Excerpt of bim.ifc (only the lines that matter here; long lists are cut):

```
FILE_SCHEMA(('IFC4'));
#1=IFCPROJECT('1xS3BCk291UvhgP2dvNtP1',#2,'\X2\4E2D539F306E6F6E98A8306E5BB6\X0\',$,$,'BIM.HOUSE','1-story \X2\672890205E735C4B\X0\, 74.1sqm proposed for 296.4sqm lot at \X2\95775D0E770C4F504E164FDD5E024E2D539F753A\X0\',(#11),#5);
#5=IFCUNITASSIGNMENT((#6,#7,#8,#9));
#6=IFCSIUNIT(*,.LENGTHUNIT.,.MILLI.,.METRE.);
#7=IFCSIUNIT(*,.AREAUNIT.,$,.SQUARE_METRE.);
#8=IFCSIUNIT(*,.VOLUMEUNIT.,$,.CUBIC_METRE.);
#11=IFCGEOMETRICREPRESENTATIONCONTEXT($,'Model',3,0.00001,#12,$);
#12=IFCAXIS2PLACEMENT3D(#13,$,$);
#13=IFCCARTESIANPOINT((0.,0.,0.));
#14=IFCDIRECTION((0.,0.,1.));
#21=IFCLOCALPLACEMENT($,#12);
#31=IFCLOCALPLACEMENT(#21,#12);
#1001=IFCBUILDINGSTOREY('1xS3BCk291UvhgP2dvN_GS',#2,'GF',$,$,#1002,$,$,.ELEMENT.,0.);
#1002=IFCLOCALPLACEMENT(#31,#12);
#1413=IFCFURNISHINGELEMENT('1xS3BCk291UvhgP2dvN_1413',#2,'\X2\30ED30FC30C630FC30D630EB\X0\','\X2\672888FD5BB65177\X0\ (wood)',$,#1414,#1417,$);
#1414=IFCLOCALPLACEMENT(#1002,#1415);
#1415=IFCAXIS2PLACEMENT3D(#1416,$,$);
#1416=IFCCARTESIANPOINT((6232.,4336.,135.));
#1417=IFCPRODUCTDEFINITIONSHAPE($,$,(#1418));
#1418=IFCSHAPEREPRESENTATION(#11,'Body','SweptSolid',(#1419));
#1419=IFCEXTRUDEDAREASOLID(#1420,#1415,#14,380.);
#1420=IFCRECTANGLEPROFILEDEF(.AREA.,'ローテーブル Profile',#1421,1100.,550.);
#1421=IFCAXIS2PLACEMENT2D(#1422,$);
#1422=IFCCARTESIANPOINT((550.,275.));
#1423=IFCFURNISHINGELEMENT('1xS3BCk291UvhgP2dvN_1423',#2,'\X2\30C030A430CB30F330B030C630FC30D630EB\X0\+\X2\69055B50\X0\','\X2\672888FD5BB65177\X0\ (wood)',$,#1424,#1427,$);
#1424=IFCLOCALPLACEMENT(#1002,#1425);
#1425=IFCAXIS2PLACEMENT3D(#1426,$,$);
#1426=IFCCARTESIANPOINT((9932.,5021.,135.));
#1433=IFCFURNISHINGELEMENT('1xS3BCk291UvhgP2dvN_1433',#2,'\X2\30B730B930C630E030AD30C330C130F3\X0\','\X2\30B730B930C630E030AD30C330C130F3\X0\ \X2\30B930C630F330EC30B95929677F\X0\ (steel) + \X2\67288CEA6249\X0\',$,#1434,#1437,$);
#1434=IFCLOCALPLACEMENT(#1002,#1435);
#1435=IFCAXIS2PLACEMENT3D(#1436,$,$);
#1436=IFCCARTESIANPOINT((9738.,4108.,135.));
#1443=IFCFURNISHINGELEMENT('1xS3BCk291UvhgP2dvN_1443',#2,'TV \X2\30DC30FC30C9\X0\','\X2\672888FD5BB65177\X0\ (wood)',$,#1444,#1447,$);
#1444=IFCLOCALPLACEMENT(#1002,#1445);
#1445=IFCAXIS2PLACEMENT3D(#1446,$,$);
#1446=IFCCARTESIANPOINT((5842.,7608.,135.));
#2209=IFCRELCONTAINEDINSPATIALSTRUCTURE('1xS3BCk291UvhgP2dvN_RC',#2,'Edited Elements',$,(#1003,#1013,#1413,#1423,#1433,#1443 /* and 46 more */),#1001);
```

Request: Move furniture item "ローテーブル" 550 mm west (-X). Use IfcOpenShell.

```python
import ifcopenshell
import ifcopenshell.api.geometry
import ifcopenshell.util.placement
import ifcopenshell.util.unit

model = ifcopenshell.open("bim.ifc")
unit_scale = ifcopenshell.util.unit.calculate_unit_scale(model)

item = model.by_id(1413)
matrix = ifcopenshell.util.placement.get_local_placement(item.ObjectPlacement)
matrix[0, 3] -= 0.55 / unit_scale
ifcopenshell.api.geometry.edit_object_placement(model, product=item, matrix=matrix, is_si=False)

print(ifcopenshell.util.placement.get_local_placement(item.ObjectPlacement).round(3) + 0.0)

model.write("bim_rev.ifc")
```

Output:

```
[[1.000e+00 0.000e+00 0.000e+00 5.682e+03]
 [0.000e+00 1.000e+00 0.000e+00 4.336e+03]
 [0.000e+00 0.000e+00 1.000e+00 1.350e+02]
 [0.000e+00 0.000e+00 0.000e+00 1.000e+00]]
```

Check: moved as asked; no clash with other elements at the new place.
